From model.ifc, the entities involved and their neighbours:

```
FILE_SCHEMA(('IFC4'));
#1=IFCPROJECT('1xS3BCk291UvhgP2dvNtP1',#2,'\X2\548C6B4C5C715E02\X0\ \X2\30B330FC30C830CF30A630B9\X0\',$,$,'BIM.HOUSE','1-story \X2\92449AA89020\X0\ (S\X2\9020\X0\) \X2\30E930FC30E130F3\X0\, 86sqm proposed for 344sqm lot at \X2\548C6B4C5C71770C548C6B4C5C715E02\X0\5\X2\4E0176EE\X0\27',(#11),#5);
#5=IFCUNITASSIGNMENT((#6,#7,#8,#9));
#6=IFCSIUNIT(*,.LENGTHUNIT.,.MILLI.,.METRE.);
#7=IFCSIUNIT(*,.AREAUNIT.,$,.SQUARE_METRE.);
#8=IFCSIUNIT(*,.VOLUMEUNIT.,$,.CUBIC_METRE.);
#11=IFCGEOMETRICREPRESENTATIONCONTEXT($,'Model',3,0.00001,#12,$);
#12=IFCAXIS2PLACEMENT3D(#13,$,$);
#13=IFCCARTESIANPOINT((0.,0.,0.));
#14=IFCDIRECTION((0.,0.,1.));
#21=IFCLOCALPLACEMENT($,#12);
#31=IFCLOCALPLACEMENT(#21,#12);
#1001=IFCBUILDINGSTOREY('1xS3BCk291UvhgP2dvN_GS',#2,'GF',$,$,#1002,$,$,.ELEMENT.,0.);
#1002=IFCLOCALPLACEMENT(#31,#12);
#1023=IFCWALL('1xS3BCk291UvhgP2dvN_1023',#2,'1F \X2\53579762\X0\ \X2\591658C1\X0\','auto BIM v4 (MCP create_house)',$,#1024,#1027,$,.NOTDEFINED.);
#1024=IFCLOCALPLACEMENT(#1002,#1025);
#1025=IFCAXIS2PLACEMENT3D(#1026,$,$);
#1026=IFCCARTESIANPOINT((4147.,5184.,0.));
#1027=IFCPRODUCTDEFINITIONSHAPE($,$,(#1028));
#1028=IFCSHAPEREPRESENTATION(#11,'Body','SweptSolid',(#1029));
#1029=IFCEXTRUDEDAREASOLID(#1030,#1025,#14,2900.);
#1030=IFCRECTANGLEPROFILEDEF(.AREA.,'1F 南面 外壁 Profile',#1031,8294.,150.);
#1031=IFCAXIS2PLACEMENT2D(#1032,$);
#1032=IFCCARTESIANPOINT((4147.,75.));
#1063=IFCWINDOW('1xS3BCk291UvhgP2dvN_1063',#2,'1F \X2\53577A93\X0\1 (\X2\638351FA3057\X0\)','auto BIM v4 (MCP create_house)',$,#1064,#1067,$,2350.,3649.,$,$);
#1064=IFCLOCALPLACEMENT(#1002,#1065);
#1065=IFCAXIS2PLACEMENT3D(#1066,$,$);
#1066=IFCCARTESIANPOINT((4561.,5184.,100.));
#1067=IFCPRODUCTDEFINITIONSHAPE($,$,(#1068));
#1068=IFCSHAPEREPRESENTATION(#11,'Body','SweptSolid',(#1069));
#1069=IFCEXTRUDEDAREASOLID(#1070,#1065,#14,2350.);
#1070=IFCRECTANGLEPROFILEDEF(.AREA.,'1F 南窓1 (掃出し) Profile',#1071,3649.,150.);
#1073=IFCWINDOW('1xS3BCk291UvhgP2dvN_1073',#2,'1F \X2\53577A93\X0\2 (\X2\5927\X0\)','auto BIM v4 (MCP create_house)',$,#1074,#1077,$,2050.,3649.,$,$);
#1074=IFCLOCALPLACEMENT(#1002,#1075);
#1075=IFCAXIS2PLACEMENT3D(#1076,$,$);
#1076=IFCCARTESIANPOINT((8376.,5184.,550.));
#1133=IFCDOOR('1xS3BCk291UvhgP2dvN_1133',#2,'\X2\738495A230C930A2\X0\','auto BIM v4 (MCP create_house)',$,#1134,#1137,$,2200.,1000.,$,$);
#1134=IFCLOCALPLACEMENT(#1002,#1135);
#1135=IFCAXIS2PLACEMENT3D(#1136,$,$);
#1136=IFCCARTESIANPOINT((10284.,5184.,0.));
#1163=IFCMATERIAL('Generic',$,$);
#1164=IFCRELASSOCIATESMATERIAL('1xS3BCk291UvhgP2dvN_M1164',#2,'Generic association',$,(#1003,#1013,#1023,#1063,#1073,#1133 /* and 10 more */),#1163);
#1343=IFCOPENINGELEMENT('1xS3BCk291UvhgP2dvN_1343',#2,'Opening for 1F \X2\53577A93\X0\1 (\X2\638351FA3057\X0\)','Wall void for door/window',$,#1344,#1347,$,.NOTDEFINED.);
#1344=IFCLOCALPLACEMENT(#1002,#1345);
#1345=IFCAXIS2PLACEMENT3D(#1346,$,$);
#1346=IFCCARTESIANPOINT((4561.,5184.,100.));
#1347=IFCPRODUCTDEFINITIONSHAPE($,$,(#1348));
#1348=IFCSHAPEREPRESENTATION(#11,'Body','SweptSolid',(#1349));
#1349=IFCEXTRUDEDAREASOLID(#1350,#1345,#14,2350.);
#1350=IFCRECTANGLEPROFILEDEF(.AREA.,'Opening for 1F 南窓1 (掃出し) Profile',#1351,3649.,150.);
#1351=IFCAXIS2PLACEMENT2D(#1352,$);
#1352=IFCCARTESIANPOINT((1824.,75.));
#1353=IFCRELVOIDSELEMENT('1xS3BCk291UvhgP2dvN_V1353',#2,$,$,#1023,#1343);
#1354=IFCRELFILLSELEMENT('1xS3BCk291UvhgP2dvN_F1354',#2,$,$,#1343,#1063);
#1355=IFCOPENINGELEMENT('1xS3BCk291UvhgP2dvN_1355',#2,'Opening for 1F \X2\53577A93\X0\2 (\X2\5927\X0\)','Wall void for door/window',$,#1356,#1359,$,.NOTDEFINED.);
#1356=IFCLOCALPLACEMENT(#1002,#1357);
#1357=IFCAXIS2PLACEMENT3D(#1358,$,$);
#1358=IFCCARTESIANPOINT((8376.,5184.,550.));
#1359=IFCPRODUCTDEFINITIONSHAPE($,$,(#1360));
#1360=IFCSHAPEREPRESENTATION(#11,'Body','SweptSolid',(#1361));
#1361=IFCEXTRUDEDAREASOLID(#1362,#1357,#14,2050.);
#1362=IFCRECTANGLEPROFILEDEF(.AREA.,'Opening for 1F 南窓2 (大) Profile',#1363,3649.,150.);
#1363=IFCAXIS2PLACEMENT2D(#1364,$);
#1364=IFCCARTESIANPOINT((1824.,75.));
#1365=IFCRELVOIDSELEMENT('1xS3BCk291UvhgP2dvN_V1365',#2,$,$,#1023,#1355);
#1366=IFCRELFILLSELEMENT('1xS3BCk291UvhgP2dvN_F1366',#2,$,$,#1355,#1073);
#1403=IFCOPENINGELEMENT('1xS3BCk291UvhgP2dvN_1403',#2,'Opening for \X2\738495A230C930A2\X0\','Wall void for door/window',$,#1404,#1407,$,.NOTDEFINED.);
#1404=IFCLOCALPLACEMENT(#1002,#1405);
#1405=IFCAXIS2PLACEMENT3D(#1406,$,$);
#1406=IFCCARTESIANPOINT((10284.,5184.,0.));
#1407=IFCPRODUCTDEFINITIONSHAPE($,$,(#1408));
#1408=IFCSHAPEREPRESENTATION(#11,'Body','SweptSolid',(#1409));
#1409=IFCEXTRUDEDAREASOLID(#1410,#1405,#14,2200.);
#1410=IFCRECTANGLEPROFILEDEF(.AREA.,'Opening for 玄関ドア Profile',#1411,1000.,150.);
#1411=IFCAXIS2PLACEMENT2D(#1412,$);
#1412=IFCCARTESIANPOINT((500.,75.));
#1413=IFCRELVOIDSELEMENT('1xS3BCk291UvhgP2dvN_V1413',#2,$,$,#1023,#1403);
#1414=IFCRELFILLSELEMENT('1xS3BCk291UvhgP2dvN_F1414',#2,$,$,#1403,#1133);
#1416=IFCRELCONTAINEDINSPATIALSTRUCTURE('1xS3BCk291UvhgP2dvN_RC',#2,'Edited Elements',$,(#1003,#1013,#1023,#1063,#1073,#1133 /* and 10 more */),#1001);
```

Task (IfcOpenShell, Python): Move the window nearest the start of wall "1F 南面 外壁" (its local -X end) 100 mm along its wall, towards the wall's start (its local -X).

```python
import ifcopenshell
import ifcopenshell.api.geometry
import ifcopenshell.util.placement
import ifcopenshell.util.unit

model = ifcopenshell.open("model.ifc")
unit_scale = ifcopenshell.util.unit.calculate_unit_scale(model)

window = model.by_guid("1xS3BCk291UvhgP2dvN_1063")
opening = window.FillsVoids[0].RelatingOpeningElement
wall = opening.VoidsElements[0].RelatingBuildingElement

wall_matrix = ifcopenshell.util.placement.get_local_placement(wall.ObjectPlacement)
shift = wall_matrix[:3, 0] * -0.1 / unit_scale
before = ifcopenshell.util.placement.get_local_placement(window.ObjectPlacement)[:3, 3].copy()

# The window is not placed relative to its opening, so move both.
for product in (opening, window):
    matrix = ifcopenshell.util.placement.get_local_placement(product.ObjectPlacement)
    matrix[:3, 3] += shift
    ifcopenshell.api.geometry.edit_object_placement(model, product=product, matrix=matrix, is_si=False)

after = ifcopenshell.util.placement.get_local_placement(window.ObjectPlacement)[:3, 3]
print("window moved by", (after - before).round(3) + 0.0)

model.write("model_rev.ifc")
```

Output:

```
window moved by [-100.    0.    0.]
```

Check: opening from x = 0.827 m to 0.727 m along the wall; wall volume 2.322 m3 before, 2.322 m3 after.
